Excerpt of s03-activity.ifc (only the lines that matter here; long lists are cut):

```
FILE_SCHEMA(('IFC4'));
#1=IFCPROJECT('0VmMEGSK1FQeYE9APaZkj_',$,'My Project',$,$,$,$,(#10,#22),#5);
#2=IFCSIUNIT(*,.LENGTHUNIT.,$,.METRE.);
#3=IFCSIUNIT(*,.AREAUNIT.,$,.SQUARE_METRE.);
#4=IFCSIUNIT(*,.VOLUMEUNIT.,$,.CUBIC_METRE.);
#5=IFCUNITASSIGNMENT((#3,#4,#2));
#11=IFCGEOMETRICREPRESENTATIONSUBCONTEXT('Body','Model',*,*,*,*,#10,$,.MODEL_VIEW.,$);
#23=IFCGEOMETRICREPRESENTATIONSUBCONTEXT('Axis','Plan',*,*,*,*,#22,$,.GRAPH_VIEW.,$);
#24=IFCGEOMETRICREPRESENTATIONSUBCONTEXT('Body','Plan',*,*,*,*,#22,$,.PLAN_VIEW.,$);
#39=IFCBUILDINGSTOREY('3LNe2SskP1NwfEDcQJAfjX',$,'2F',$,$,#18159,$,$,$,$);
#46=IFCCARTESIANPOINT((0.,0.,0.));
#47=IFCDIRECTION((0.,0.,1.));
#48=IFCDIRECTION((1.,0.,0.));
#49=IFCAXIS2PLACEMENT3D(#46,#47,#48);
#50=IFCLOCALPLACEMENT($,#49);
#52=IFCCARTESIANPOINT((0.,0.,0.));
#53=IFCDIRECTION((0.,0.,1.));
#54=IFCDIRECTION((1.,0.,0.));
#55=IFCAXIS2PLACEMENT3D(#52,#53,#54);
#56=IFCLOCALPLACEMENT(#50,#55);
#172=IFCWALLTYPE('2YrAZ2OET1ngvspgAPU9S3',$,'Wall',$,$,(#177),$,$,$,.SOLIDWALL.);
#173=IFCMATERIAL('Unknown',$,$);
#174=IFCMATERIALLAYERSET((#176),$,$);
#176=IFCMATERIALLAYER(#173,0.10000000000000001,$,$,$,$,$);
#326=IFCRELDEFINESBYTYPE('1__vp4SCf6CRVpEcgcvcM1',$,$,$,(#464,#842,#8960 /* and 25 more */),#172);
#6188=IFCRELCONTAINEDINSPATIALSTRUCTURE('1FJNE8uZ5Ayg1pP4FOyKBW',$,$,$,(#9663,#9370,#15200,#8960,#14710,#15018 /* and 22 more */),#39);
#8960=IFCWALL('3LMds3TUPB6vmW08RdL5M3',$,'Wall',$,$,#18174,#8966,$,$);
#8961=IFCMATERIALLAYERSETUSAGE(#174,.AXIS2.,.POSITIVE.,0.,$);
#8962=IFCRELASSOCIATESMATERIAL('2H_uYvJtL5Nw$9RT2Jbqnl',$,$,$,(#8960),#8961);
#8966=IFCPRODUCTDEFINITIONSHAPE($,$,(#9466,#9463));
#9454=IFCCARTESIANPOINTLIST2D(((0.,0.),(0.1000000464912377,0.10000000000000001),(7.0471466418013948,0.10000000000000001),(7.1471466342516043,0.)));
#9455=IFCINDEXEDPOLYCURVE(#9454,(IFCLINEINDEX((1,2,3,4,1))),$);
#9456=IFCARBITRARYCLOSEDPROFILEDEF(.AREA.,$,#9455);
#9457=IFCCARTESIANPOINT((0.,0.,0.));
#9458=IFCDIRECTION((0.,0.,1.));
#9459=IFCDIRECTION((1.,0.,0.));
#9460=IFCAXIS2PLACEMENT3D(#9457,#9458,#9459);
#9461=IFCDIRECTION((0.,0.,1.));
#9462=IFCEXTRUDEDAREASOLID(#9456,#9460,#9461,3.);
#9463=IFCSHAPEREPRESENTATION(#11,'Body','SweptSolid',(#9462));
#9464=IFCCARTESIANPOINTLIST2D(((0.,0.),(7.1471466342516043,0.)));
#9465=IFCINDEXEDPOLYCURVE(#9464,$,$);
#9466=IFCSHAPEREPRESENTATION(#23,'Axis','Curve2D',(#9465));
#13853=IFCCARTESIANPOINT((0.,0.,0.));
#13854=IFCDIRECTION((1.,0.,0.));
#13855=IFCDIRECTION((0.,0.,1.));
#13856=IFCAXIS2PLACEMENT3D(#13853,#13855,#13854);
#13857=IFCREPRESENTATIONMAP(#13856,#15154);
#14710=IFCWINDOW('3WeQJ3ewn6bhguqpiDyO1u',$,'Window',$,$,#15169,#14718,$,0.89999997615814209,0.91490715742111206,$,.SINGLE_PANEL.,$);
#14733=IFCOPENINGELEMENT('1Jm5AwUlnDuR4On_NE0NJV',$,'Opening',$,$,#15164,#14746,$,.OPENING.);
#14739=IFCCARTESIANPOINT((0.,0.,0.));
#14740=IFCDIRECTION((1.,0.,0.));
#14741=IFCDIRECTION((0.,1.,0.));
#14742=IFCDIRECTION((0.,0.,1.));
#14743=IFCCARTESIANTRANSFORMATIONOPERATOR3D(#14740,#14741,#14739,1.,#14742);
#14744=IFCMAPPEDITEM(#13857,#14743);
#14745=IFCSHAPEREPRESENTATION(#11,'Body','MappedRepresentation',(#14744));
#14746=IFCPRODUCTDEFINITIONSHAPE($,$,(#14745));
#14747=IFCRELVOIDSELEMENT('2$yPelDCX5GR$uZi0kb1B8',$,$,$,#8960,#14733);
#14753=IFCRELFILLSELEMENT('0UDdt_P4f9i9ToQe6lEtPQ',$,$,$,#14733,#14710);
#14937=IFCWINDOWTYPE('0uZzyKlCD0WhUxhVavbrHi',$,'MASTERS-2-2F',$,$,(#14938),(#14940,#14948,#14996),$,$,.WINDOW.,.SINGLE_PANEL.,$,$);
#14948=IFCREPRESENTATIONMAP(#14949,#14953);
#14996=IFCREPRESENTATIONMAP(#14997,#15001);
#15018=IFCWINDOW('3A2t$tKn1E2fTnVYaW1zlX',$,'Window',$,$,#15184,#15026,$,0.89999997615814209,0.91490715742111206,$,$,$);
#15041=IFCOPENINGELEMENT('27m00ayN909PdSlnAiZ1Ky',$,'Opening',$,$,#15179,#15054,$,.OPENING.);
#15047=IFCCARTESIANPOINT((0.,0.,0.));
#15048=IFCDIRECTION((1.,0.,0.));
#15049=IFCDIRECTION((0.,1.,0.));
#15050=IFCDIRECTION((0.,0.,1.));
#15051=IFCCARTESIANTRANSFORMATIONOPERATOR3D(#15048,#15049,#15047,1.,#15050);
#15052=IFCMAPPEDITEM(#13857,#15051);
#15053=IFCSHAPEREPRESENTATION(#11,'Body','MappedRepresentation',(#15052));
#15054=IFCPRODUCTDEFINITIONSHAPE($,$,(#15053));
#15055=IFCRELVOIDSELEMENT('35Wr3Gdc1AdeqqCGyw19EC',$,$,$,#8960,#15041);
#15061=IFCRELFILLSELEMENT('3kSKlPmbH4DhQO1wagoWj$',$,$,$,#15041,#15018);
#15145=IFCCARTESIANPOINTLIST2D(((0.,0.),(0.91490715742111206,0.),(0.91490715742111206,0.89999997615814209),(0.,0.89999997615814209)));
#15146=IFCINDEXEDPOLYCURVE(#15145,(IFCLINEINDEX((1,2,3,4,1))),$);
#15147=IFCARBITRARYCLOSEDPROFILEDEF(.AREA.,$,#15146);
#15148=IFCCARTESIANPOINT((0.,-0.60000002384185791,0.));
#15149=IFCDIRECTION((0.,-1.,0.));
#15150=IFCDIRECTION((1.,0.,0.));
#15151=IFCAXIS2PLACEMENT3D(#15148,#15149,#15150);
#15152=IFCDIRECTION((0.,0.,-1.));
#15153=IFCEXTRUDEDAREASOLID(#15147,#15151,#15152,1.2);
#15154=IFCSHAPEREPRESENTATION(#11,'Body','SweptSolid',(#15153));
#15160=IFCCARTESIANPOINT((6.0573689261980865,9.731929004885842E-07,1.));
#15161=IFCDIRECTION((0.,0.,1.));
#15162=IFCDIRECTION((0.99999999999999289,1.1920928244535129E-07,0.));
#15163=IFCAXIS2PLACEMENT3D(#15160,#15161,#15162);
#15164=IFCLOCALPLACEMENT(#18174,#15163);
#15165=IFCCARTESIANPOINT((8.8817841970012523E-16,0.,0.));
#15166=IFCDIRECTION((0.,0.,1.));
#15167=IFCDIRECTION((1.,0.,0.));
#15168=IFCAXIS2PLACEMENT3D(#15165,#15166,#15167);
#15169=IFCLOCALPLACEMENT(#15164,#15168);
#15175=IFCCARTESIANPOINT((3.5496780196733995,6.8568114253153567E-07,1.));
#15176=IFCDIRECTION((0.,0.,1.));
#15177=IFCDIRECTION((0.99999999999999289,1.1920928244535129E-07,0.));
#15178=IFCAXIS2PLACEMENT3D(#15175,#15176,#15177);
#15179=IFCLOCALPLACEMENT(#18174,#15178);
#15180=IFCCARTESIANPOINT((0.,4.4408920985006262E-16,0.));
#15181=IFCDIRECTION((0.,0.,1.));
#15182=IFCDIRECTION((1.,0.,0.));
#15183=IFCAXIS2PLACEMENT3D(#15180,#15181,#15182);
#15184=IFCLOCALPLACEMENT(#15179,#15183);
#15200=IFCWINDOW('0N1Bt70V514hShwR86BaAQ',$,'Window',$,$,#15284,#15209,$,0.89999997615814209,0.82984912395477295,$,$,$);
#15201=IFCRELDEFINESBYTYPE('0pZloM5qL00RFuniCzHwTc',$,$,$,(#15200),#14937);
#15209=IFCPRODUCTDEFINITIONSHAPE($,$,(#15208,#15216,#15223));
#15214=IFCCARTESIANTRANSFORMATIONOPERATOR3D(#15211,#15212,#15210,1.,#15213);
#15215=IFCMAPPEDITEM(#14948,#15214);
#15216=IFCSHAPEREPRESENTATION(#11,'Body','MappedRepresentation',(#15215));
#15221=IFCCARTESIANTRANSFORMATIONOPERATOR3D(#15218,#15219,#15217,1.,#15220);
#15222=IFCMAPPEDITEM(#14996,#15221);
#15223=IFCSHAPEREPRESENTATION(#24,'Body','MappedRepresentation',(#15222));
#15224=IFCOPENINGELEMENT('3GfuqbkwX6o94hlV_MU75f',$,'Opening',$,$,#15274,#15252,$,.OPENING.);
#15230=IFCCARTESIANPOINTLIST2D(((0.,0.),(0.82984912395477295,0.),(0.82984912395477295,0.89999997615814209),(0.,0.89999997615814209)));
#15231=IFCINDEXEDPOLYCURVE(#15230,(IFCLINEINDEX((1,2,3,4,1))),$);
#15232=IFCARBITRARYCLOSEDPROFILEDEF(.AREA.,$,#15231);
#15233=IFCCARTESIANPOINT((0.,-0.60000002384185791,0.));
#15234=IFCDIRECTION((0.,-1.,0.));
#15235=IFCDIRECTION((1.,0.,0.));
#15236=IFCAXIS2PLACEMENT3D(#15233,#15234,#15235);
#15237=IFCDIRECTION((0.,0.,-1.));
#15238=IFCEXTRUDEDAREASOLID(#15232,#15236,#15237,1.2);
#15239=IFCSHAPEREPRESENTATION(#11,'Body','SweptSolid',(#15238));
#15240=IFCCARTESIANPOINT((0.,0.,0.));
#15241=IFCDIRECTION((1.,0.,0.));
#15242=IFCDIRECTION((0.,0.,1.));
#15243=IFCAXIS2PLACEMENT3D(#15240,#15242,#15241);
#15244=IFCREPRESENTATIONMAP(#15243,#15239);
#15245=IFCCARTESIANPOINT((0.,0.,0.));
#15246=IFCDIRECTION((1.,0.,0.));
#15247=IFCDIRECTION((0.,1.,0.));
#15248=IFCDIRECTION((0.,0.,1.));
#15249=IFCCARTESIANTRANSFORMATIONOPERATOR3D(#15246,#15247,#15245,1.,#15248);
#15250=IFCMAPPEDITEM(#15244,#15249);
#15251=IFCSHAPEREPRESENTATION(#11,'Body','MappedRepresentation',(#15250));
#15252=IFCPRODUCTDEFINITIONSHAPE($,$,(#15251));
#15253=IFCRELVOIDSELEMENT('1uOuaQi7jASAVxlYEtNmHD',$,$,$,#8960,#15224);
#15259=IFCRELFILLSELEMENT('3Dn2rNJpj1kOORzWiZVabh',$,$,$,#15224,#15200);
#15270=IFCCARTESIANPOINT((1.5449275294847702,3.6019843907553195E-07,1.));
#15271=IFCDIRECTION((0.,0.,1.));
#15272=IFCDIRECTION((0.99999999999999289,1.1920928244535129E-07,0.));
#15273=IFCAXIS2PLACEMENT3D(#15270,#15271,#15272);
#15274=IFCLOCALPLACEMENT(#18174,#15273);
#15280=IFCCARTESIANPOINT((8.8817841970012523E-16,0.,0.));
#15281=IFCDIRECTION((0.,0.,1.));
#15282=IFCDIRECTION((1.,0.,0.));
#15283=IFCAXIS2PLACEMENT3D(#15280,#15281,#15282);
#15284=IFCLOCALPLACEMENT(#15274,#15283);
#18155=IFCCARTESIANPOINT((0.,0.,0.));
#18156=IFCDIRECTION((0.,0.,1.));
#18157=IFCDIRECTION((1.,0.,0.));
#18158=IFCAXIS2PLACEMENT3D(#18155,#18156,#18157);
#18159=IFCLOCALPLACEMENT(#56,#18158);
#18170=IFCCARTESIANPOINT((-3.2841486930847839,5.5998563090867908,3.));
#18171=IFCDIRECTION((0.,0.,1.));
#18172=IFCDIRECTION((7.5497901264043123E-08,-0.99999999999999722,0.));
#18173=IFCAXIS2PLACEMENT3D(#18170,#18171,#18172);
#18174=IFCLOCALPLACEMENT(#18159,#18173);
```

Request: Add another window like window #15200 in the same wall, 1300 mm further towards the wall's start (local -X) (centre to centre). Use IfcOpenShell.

```python
import ifcopenshell
import ifcopenshell.api.feature
import ifcopenshell.api.geometry
import ifcopenshell.api.root
import ifcopenshell.geom
import ifcopenshell.util.element
import ifcopenshell.util.placement
import ifcopenshell.util.shape

model = ifcopenshell.open("s03-activity.ifc")
settings = ifcopenshell.geom.settings()


def volume(element):
    """Net volume in cubic metres, openings subtracted."""
    shape = ifcopenshell.geom.create_shape(settings, element)
    return ifcopenshell.util.shape.get_volume(shape.geometry)


window = model.by_guid("0N1Bt70V514hShwR86BaAQ")
opening = window.FillsVoids[0].RelatingOpeningElement
wall = opening.VoidsElements[0].RelatingBuildingElement
before = volume(wall)
shift = ifcopenshell.util.placement.get_local_placement(wall.ObjectPlacement)[:3, 0] * -1.3

# copy_class copies the void relationship, type, container and properties, but no geometry.
new_opening = ifcopenshell.api.root.copy_class(model, product=opening)
new_opening.Representation = ifcopenshell.util.element.copy_deep(
    model, opening.Representation, exclude=["IfcGeometricRepresentationContext", "IfcRepresentationMap"]
)
new_window = ifcopenshell.api.root.copy_class(model, product=window)
new_window.Representation = ifcopenshell.util.element.copy_deep(
    model, window.Representation, exclude=["IfcGeometricRepresentationContext", "IfcRepresentationMap"]
)
ifcopenshell.api.feature.add_filling(model, opening=new_opening, element=new_window)

for old, new in ((opening, new_opening), (window, new_window)):
    matrix = ifcopenshell.util.placement.get_local_placement(old.ObjectPlacement)
    matrix[:3, 3] += shift
    ifcopenshell.api.geometry.edit_object_placement(model, product=new, matrix=matrix, is_si=False)

after = volume(wall)

print(f"wall volume {before:.3f} -> {after:.3f} m3")

model.write("s03-activity-out.ifc")
```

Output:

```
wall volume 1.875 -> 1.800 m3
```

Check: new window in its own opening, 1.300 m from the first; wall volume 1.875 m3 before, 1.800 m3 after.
